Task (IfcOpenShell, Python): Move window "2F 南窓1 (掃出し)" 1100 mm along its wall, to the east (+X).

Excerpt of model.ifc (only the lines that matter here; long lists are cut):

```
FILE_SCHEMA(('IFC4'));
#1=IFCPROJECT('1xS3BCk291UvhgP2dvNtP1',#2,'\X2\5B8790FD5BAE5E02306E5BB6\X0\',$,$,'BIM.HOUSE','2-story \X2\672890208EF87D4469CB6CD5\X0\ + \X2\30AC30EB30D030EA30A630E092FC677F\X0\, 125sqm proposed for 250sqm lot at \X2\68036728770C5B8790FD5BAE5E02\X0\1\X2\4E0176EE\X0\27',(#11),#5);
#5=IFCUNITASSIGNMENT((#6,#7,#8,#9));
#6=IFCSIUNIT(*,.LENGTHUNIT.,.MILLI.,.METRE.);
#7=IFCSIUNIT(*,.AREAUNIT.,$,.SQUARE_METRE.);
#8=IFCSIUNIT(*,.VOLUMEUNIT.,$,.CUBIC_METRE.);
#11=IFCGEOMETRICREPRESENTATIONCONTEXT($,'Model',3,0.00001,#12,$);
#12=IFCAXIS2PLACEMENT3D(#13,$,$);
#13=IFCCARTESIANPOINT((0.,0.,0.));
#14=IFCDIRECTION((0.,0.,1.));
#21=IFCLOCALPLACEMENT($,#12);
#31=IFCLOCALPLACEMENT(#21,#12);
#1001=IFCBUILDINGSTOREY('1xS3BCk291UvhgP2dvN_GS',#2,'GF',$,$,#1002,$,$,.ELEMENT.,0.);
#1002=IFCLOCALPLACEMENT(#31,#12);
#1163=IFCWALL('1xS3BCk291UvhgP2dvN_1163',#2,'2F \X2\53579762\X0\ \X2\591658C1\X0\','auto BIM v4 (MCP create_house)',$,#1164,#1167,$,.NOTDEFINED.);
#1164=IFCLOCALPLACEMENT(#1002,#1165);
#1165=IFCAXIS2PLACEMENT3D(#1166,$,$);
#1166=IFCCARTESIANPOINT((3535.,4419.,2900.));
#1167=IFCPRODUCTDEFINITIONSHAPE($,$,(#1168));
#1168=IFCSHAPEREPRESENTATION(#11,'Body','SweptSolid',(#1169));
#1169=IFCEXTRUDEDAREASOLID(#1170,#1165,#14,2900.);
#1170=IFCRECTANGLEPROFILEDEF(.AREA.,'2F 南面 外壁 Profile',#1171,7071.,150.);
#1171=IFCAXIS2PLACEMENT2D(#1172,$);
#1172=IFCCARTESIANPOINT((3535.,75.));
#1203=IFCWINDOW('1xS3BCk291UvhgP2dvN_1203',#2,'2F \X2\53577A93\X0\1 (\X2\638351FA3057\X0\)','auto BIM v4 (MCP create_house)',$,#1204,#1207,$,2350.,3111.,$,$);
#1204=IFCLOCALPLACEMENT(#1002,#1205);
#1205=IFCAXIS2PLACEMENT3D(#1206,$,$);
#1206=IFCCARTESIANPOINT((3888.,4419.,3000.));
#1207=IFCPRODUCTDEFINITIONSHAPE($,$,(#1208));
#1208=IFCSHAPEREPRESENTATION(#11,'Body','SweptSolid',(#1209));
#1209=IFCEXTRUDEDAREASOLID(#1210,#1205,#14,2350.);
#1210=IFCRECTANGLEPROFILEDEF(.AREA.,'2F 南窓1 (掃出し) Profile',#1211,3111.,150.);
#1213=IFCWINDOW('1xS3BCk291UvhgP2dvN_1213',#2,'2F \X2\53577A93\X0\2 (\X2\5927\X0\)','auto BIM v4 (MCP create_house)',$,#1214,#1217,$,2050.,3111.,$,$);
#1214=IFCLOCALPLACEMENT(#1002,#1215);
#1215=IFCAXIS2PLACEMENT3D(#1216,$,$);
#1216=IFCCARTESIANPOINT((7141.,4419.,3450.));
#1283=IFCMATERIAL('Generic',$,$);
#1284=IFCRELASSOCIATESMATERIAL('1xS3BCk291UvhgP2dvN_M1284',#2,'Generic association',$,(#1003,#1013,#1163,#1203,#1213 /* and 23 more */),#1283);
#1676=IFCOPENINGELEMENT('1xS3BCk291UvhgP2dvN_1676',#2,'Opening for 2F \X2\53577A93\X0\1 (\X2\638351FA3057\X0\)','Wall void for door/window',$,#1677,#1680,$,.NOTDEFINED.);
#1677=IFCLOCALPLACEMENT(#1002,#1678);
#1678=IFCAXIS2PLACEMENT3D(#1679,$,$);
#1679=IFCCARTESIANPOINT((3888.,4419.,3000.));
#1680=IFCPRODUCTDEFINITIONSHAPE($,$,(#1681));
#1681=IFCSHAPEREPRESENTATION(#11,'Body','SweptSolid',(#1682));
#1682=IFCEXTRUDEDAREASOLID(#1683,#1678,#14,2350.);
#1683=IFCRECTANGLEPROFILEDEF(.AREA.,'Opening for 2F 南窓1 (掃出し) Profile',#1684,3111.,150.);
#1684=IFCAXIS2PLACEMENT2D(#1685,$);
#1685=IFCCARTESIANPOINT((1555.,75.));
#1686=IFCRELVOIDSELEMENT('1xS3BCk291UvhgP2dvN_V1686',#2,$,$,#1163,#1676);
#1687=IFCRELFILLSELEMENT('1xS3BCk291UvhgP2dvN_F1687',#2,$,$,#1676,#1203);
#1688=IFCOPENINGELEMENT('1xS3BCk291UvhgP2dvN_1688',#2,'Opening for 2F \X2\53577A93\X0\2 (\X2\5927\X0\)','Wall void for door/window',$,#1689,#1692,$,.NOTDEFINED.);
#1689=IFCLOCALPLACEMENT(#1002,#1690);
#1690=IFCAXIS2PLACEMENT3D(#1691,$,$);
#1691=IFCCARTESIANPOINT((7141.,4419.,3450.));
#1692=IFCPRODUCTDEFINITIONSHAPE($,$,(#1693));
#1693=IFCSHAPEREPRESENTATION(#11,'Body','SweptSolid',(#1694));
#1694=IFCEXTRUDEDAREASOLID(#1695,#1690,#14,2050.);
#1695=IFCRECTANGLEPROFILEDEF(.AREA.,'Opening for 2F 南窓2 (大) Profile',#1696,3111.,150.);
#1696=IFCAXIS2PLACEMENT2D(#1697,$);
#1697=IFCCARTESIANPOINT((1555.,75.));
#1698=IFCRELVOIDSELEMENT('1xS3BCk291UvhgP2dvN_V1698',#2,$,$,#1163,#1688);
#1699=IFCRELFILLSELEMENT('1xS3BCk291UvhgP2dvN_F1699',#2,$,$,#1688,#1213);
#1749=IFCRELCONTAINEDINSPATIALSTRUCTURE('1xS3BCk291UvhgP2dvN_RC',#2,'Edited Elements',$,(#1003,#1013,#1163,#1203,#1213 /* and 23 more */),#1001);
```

```python
import ifcopenshell
import ifcopenshell.api.geometry
import ifcopenshell.util.placement
import ifcopenshell.util.unit

model = ifcopenshell.open("model.ifc")
unit_scale = ifcopenshell.util.unit.calculate_unit_scale(model)

window = model.by_guid("1xS3BCk291UvhgP2dvN_1203")
opening = window.FillsVoids[0].RelatingOpeningElement
wall = opening.VoidsElements[0].RelatingBuildingElement

wall_matrix = ifcopenshell.util.placement.get_local_placement(wall.ObjectPlacement)
shift = wall_matrix[:3, 0] * 1.1 / unit_scale
before = ifcopenshell.util.placement.get_local_placement(window.ObjectPlacement)[:3, 3].copy()

# The window is not placed relative to its opening, so move both.
for product in (opening, window):
    matrix = ifcopenshell.util.placement.get_local_placement(product.ObjectPlacement)
    matrix[:3, 3] += shift
    ifcopenshell.api.geometry.edit_object_placement(model, product=product, matrix=matrix, is_si=False)

after = ifcopenshell.util.placement.get_local_placement(window.ObjectPlacement)[:3, 3]
print("window moved by", (after - before).round(3) + 0.0)

model.write("model_updated.ifc")
```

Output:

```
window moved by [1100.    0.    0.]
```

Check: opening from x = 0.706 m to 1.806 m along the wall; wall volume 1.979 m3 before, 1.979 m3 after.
